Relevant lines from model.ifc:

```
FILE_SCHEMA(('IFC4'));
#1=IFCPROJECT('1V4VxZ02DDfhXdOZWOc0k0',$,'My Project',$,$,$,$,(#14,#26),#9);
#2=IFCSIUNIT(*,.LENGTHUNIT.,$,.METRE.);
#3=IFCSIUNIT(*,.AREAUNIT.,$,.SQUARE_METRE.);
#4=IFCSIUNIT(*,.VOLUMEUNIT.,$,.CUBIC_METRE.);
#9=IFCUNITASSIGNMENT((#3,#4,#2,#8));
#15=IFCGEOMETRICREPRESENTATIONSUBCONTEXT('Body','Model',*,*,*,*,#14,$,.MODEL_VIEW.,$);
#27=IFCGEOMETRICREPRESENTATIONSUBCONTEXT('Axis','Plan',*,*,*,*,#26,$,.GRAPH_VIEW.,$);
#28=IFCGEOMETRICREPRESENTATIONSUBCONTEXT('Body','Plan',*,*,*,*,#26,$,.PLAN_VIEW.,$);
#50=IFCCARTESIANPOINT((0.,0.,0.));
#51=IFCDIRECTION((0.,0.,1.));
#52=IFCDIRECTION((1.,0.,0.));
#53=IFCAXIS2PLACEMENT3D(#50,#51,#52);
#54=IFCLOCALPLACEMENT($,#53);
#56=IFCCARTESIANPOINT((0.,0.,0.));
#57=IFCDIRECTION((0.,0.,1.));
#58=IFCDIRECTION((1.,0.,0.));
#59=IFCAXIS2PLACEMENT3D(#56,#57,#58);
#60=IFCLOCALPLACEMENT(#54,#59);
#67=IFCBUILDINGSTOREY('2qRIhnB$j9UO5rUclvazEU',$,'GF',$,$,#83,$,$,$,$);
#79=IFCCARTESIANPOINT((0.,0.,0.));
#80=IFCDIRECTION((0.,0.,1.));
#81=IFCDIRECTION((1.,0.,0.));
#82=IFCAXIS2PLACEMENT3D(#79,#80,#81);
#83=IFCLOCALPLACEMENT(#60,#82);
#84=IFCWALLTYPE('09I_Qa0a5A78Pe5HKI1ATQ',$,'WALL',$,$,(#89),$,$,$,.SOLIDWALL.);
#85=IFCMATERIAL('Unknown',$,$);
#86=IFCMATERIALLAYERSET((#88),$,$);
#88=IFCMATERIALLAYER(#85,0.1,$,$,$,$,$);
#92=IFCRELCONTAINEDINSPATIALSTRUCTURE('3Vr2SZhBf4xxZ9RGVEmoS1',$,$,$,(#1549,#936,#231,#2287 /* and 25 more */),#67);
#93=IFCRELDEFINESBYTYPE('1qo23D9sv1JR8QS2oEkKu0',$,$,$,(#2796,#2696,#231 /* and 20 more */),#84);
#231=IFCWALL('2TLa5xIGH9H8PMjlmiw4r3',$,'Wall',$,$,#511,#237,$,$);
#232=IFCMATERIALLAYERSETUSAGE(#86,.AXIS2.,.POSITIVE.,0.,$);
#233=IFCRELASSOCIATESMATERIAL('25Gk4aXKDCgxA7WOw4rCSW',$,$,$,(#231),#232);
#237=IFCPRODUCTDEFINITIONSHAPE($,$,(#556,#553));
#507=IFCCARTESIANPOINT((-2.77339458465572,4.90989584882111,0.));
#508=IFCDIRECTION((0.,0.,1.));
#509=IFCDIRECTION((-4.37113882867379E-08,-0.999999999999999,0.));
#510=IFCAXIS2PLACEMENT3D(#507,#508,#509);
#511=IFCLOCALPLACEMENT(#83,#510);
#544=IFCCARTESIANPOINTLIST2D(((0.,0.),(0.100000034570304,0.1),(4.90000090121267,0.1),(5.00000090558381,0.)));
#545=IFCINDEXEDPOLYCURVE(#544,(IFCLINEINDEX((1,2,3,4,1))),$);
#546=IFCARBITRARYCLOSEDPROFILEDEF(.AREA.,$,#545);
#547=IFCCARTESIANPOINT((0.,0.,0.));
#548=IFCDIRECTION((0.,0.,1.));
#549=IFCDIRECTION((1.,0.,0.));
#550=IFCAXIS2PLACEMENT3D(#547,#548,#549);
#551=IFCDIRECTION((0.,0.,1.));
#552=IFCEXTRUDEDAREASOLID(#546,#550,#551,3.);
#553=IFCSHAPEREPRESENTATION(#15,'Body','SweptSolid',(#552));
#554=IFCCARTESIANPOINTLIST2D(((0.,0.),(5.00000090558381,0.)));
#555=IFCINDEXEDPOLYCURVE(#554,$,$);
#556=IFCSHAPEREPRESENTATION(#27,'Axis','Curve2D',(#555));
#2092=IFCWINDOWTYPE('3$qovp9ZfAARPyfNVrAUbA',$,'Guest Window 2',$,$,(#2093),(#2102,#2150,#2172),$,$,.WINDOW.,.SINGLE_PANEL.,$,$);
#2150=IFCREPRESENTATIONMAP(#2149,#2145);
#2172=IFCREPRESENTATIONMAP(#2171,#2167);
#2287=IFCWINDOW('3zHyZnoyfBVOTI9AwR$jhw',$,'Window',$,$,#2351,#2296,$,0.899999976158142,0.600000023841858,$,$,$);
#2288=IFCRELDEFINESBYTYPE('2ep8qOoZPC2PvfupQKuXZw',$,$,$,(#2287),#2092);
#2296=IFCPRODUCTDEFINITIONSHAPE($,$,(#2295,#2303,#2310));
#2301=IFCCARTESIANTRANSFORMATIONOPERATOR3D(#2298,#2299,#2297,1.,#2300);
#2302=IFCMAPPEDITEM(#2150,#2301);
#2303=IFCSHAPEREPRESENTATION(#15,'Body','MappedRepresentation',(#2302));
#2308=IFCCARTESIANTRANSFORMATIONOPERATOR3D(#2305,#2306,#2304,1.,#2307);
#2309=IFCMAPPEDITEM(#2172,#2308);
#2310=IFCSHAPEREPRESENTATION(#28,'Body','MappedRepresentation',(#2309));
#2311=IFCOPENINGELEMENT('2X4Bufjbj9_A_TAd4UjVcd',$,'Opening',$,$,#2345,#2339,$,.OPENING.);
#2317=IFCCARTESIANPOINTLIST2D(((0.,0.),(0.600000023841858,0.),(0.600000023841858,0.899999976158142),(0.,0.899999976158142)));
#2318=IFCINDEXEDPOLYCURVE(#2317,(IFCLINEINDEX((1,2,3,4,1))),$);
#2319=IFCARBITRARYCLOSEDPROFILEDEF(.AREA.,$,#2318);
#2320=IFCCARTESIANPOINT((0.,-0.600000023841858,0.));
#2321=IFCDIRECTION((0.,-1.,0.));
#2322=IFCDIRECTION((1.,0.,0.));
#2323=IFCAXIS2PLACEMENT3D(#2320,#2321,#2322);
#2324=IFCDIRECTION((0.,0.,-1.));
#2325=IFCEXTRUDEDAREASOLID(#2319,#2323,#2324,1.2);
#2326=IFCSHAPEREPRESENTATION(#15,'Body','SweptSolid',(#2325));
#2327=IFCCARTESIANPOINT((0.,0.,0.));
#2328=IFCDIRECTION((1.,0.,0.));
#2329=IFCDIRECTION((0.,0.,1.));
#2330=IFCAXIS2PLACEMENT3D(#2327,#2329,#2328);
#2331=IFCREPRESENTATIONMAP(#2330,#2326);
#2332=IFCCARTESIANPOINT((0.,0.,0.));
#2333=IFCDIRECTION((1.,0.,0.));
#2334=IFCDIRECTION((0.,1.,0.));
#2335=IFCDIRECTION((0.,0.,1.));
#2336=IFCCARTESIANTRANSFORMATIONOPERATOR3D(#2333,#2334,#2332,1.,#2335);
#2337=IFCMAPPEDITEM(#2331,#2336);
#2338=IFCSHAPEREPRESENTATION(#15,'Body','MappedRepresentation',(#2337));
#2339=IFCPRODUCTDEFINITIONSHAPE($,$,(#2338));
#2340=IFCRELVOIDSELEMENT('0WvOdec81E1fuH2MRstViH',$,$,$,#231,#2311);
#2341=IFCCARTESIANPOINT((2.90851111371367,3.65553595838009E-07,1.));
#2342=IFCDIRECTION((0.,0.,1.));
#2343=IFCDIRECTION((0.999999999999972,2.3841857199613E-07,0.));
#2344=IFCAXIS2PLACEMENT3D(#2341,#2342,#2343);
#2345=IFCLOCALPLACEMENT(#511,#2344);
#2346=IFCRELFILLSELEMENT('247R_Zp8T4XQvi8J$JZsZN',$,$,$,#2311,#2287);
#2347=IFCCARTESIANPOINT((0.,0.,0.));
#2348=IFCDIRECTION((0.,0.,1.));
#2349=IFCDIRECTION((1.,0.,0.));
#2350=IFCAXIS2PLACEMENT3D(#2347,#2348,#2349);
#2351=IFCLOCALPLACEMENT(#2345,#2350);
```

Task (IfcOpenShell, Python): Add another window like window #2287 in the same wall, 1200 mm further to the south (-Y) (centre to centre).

```python
import ifcopenshell
import ifcopenshell.api.feature
import ifcopenshell.api.geometry
import ifcopenshell.api.root
import ifcopenshell.geom
import ifcopenshell.util.element
import ifcopenshell.util.placement
import ifcopenshell.util.shape

model = ifcopenshell.open("model.ifc")
settings = ifcopenshell.geom.settings()


def volume(element):
    """Net volume in cubic metres, openings subtracted."""
    shape = ifcopenshell.geom.create_shape(settings, element)
    return ifcopenshell.util.shape.get_volume(shape.geometry)


window = model.by_guid("3zHyZnoyfBVOTI9AwR$jhw")
opening = window.FillsVoids[0].RelatingOpeningElement
wall = opening.VoidsElements[0].RelatingBuildingElement
before = volume(wall)
shift = ifcopenshell.util.placement.get_local_placement(wall.ObjectPlacement)[:3, 0] * 1.2

# copy_class copies the void relationship, type, container and properties, but no geometry.
new_opening = ifcopenshell.api.root.copy_class(model, product=opening)
new_opening.Representation = ifcopenshell.util.element.copy_deep(
    model, opening.Representation, exclude=["IfcGeometricRepresentationContext", "IfcRepresentationMap"]
)
new_window = ifcopenshell.api.root.copy_class(model, product=window)
new_window.Representation = ifcopenshell.util.element.copy_deep(
    model, window.Representation, exclude=["IfcGeometricRepresentationContext", "IfcRepresentationMap"]
)
ifcopenshell.api.feature.add_filling(model, opening=new_opening, element=new_window)

for old, new in ((opening, new_opening), (window, new_window)):
    matrix = ifcopenshell.util.placement.get_local_placement(old.ObjectPlacement)
    matrix[:3, 3] += shift
    ifcopenshell.api.geometry.edit_object_placement(model, product=new, matrix=matrix, is_si=False)

after = volume(wall)

print(f"wall volume {before:.3f} -> {after:.3f} m3")

model.write("model_rev.ifc")
```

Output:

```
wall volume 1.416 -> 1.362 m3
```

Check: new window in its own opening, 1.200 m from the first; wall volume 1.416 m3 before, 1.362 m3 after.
